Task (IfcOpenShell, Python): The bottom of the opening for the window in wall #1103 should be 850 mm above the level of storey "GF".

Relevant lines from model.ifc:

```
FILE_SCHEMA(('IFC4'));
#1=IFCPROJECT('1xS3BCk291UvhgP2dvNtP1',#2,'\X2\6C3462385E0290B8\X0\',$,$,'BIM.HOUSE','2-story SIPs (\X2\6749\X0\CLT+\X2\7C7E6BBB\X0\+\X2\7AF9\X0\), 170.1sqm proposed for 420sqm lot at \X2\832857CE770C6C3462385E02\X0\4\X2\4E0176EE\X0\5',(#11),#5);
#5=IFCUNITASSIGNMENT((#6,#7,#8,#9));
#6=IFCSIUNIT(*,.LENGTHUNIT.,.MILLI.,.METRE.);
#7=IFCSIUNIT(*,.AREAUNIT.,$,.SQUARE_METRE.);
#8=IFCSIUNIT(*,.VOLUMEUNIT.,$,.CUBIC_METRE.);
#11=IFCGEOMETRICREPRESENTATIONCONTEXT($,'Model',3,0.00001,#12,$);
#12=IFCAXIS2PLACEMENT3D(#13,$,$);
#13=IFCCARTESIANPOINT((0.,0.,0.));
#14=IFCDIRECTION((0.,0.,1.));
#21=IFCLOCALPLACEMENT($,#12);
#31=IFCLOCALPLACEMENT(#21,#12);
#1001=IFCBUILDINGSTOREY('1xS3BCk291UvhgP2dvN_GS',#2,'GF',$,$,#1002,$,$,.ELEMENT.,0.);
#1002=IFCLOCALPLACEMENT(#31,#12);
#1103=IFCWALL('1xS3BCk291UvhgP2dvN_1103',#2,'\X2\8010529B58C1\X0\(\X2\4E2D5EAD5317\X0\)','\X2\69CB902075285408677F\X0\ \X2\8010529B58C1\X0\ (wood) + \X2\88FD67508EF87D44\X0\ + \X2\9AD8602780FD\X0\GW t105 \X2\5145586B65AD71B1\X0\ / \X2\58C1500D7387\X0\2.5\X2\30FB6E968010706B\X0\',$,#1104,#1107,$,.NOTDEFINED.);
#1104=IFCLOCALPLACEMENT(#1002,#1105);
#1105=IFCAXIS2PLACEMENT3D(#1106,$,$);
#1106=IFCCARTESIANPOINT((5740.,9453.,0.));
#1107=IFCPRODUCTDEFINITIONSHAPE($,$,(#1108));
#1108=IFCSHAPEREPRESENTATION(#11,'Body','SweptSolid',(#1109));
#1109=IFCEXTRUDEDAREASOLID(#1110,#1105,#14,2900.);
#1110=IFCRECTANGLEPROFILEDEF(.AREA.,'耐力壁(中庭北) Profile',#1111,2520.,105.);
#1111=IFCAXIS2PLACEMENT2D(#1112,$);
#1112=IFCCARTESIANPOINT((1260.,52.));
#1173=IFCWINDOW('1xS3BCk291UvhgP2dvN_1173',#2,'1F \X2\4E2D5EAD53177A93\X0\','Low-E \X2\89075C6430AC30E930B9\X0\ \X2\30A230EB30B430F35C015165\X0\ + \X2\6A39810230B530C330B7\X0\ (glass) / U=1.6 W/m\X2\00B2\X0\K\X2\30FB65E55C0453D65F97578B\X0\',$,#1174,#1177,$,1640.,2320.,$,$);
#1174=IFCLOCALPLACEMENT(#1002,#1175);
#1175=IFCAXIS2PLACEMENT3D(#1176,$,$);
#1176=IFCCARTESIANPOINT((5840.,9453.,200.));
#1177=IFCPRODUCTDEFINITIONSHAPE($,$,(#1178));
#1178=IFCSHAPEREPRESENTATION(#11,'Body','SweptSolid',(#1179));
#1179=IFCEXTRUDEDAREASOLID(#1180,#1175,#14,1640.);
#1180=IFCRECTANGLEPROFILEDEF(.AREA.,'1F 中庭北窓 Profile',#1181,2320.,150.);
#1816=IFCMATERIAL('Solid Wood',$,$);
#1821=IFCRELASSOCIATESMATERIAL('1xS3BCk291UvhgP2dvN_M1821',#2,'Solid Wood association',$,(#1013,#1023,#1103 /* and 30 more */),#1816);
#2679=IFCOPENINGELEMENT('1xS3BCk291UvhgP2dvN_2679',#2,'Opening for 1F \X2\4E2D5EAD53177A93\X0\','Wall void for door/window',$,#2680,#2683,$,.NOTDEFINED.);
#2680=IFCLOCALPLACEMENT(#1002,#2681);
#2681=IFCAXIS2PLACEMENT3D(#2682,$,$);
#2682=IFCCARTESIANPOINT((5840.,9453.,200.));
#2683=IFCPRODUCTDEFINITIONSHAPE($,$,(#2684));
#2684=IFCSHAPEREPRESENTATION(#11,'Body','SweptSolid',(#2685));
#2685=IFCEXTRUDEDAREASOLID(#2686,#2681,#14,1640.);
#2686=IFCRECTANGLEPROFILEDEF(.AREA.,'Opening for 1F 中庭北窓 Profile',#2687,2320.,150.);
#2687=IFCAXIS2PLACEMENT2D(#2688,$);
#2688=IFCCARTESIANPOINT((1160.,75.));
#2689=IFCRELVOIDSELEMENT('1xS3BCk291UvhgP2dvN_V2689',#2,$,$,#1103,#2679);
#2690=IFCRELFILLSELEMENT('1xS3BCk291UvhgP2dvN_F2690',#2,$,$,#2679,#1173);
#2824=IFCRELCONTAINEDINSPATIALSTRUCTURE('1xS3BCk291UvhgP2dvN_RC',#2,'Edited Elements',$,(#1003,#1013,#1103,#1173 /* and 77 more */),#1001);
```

```python
import numpy as np
import ifcopenshell
import ifcopenshell.api.geometry
import ifcopenshell.geom
import ifcopenshell.util.element
import ifcopenshell.util.placement
import ifcopenshell.util.shape
import ifcopenshell.util.unit

model = ifcopenshell.open("model.ifc")
unit_scale = ifcopenshell.util.unit.calculate_unit_scale(model)

window = model.by_id(1173)
opening = window.FillsVoids[0].RelatingOpeningElement
storey = ifcopenshell.util.element.get_container(window, ifc_class="IfcBuildingStorey")
level = ifcopenshell.util.placement.get_local_placement(storey.ObjectPlacement)[2, 3]

# The opening's origin need not be at the sill, so measure its lowest point.
shape = ifcopenshell.geom.create_shape(ifcopenshell.geom.settings(), opening)
bottom = ifcopenshell.util.shape.get_shape_bottom_elevation(shape, shape.geometry) / unit_scale
dz = level + 0.85 / unit_scale - bottom

shift = np.array([0.0, 0.0, dz])
# The window is not placed relative to its opening, so move both.
for product in (opening, window):
    matrix = ifcopenshell.util.placement.get_local_placement(product.ObjectPlacement)
    matrix[:3, 3] += shift
    ifcopenshell.api.geometry.edit_object_placement(model, product=product, matrix=matrix, is_si=False)

print(f"moved by {dz * unit_scale:+.3f} m")

model.write("model_edited.ifc")
```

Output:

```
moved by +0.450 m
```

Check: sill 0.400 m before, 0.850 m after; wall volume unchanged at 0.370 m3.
